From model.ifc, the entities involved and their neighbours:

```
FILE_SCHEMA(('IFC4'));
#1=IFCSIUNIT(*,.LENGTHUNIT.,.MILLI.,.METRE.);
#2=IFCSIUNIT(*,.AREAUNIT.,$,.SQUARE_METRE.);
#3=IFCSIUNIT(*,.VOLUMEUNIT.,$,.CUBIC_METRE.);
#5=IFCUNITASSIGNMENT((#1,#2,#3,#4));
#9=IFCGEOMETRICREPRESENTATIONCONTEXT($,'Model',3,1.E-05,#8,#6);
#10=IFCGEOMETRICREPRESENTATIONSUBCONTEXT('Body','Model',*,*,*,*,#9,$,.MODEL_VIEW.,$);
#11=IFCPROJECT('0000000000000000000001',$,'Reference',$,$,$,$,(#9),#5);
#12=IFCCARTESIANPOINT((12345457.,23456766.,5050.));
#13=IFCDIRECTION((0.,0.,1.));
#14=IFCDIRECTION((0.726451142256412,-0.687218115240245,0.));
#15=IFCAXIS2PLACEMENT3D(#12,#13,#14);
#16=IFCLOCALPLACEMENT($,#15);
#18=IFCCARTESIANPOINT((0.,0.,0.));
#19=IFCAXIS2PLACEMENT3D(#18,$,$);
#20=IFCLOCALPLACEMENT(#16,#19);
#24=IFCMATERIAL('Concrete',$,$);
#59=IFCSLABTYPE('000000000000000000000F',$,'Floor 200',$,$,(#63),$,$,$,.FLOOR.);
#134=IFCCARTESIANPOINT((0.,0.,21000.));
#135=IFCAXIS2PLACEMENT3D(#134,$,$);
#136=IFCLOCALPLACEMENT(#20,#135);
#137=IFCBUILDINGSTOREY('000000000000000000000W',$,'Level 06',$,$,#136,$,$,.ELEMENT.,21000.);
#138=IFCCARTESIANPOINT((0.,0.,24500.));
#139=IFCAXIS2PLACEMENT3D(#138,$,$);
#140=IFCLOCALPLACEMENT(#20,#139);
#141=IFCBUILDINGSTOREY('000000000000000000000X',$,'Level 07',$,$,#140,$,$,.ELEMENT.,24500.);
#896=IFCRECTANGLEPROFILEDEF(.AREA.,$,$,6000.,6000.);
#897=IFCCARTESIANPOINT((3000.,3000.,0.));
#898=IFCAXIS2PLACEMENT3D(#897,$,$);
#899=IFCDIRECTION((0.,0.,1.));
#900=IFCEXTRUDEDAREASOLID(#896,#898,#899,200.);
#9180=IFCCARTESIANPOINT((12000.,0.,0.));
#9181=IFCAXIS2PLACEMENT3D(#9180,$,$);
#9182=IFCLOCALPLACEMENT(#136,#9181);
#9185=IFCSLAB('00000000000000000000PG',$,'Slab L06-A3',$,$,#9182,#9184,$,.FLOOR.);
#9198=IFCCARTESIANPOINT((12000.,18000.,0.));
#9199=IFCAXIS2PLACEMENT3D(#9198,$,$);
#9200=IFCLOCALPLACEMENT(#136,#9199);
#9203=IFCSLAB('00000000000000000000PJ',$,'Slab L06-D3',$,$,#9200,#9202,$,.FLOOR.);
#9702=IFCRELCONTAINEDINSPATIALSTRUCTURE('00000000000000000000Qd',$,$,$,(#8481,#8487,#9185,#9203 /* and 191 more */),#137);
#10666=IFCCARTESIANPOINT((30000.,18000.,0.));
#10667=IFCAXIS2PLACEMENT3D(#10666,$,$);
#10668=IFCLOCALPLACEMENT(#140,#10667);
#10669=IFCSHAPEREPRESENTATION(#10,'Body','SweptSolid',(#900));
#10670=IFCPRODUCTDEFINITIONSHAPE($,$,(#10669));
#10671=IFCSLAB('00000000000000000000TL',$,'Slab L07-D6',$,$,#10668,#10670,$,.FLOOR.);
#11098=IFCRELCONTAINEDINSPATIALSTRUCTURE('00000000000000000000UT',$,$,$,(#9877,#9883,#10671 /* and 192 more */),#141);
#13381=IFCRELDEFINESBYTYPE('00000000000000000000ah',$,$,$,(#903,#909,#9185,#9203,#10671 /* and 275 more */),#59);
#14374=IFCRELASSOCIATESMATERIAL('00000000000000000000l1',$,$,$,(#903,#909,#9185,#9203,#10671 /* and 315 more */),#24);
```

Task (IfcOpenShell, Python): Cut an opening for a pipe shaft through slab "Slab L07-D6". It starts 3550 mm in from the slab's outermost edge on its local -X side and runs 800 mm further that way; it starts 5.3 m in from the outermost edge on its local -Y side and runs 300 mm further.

```python
import numpy as np
import ifcopenshell
import ifcopenshell.api.feature
import ifcopenshell.api.geometry
import ifcopenshell.api.root
import ifcopenshell.geom
import ifcopenshell.util.placement
import ifcopenshell.util.representation
import ifcopenshell.util.shape
import ifcopenshell.util.unit

model = ifcopenshell.open("model.ifc")
unit_scale = ifcopenshell.util.unit.calculate_unit_scale(model)
settings = ifcopenshell.geom.settings()


def volume(element):
    """Net volume in cubic metres, openings subtracted."""
    shape = ifcopenshell.geom.create_shape(settings, element)
    return ifcopenshell.util.shape.get_volume(shape.geometry)


slab = model.by_guid("00000000000000000000TL")
before = volume(slab)

# Extent in the slab's own axes, in metres. The edges named are its -X and -Y sides.
slab_shape = ifcopenshell.geom.create_shape(settings, slab)
vertices = ifcopenshell.util.shape.get_vertices(slab_shape.geometry)
x_min, y_min, bottom = vertices.min(axis=0)
top = vertices[:, 2].max()

opening = ifcopenshell.api.root.create_entity(model, ifc_class="IfcOpeningElement", name="Pipe shaft opening", predefined_type="OPENING")
context = ifcopenshell.util.representation.get_context(model, "Model", "Body", "MODEL_VIEW")
width, depth = 0.8, 0.3
outline = [(0.0, 0.0), (width, 0.0), (width, depth), (0.0, depth), (0.0, 0.0)]
# Overshoot both faces by 50 mm so the cut is clean.
shape = ifcopenshell.api.geometry.add_slab_representation(
    model, context=context, depth=top - bottom + 0.1, polyline=outline
)
ifcopenshell.api.geometry.assign_representation(model, product=opening, representation=shape)

matrix = ifcopenshell.util.placement.get_local_placement(slab.ObjectPlacement)
matrix[:, 3] = matrix @ np.append(np.array([x_min + 3.55, y_min + 5.3, bottom - 0.05]) / unit_scale, 1.0)
ifcopenshell.api.geometry.edit_object_placement(model, product=opening, matrix=matrix, is_si=False)
ifcopenshell.api.feature.add_feature(model, feature=opening, element=slab)

after = volume(slab)

print(f"slab volume {before:.3f} -> {after:.3f} m3")

model.write("model_updated.ifc")
```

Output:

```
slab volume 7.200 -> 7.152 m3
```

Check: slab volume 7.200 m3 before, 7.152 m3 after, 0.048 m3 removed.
